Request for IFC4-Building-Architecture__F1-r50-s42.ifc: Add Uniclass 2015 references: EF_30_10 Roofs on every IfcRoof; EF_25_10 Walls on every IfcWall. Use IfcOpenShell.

First a look at what the model holds.

```python
import ifcopenshell

model = ifcopenshell.open("IFC4-Building-Architecture__F1-r50-s42.ifc")
print(model.schema)
print("classifications:", [c.Name for c in model.by_type("IfcClassification")])
for ifc_class in ("IfcDoor", "IfcRoof", "IfcStair", "IfcWall", "IfcWindow"):
    print(ifc_class, len(model.by_type(ifc_class)))
```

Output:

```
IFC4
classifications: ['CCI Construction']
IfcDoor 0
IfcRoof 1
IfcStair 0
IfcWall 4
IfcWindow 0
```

```python
import ifcopenshell
import ifcopenshell.api.classification

model = ifcopenshell.open("IFC4-Building-Architecture__F1-r50-s42.ifc")

system = ifcopenshell.api.classification.add_classification(model, classification="Uniclass 2015")

codes = {
    "IfcRoof": ("EF_30_10", "Roofs"),
    "IfcWall": ("EF_25_10", "Walls"),
}
for ifc_class, (code, name) in codes.items():
    products = model.by_type(ifc_class)
    ifcopenshell.api.classification.add_reference(
        model, products=products, classification=system, identification=code, name=name
    )
    print(code, len(products))

model.write("IFC4-Building-Architecture__F1-r50-s42-out.ifc")
```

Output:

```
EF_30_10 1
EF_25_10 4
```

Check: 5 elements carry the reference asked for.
